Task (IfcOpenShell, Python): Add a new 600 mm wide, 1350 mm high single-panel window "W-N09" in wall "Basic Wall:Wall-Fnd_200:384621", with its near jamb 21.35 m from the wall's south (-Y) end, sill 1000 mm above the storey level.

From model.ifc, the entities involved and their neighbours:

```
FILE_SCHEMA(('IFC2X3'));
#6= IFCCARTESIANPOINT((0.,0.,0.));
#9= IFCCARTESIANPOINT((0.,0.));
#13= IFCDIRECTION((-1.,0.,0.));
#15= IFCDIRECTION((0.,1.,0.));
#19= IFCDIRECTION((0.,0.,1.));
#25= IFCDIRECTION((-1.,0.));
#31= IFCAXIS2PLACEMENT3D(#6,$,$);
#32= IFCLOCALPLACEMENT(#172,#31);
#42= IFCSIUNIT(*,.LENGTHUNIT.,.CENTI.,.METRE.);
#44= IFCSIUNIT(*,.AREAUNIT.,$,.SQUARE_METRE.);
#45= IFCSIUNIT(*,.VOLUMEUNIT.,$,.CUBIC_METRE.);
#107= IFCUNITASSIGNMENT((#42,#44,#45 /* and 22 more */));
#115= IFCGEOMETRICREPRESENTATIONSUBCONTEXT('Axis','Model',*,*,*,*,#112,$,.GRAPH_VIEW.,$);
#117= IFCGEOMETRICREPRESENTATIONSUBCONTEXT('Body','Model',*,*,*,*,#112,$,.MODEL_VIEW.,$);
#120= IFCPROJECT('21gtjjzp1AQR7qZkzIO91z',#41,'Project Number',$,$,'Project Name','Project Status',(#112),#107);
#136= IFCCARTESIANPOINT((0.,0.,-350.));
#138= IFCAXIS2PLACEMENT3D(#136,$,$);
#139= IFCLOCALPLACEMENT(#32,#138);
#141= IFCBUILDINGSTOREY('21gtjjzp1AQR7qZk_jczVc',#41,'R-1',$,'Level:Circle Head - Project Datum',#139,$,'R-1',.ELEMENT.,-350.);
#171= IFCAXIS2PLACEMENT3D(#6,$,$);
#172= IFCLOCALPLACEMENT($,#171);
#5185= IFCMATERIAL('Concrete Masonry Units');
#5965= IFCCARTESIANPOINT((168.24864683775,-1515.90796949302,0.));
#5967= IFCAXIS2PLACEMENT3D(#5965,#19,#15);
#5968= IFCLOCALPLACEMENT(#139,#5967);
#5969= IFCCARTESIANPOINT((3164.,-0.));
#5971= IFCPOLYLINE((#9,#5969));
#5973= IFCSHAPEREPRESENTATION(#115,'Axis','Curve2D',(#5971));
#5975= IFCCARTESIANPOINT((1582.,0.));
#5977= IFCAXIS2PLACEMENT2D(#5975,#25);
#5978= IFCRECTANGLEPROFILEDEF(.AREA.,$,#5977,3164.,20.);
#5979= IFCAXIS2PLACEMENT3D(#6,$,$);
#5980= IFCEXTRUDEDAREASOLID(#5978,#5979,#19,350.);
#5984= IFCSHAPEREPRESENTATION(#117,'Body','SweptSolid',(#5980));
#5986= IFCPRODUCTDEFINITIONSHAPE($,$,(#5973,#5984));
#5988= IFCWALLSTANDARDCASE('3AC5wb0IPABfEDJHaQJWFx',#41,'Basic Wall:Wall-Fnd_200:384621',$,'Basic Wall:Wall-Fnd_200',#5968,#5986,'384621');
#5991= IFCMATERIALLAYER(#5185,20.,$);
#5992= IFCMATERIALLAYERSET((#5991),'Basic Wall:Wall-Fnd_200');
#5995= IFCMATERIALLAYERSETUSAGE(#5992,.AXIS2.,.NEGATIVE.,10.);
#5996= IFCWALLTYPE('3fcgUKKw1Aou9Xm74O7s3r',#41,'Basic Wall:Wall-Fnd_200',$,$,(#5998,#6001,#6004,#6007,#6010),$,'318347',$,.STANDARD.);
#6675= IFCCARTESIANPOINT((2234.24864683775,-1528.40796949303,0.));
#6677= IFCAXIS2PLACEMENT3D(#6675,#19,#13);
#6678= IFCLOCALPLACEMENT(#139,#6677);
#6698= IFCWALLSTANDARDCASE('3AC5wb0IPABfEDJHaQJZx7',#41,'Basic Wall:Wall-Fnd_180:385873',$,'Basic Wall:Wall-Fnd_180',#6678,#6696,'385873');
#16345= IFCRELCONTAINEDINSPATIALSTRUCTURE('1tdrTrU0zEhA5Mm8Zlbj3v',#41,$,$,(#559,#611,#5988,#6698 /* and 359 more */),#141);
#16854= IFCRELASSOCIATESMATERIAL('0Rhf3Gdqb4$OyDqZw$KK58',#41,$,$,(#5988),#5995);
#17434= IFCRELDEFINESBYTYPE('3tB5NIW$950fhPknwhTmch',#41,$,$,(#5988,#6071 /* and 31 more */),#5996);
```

```python
import numpy as np
import ifcopenshell
import ifcopenshell.api.feature
import ifcopenshell.api.geometry
import ifcopenshell.api.root
import ifcopenshell.api.spatial
import ifcopenshell.api.type
import ifcopenshell.geom
import ifcopenshell.util.element
import ifcopenshell.util.placement
import ifcopenshell.util.representation
import ifcopenshell.util.shape
import ifcopenshell.util.unit

model = ifcopenshell.open("model.ifc")
unit_scale = ifcopenshell.util.unit.calculate_unit_scale(model)
settings = ifcopenshell.geom.settings()


def volume(element):
    """Net volume in cubic metres, openings subtracted."""
    shape = ifcopenshell.geom.create_shape(settings, element)
    return ifcopenshell.util.shape.get_volume(shape.geometry)


wall = model.by_guid("3AC5wb0IPABfEDJHaQJWFx")
storey = ifcopenshell.util.element.get_container(wall, ifc_class="IfcBuildingStorey")
context = ifcopenshell.util.representation.get_context(model, "Model", "Body", "MODEL_VIEW")
before = volume(wall)

width, height, from_end, sill = 0.6, 1.35, 21.35, 1  # metres

# The wall runs along its own X axis, and the end named is its -X end.
wall_shape = ifcopenshell.geom.create_shape(settings, wall)
x, y, z = ifcopenshell.util.shape.get_vertices(wall_shape.geometry).T
start = x.min() + from_end
face, thickness = float(y.min()), float(y.max() - y.min())
wall_matrix = ifcopenshell.util.placement.get_local_placement(wall.ObjectPlacement)
level = ifcopenshell.util.placement.get_local_placement(storey.ObjectPlacement)[2, 3]


def in_wall(x, y):
    """Placement at x, y metres in the wall's axes, at sill height."""
    matrix = wall_matrix.copy()
    matrix[:, 3] = wall_matrix @ np.array([x / unit_scale, y / unit_scale, 0.0, 1.0])
    matrix[2, 3] = level + sill / unit_scale
    return matrix


# Opening: a box that overshoots both wall faces by 50 mm.
opening = ifcopenshell.api.root.create_entity(model, ifc_class="IfcOpeningElement")
box = ifcopenshell.api.geometry.add_wall_representation(
    model, context=context, length=width, height=height, thickness=thickness + 0.1
)
ifcopenshell.api.geometry.assign_representation(model, product=opening, representation=box)
ifcopenshell.api.geometry.edit_object_placement(model, product=opening, matrix=in_wall(start, face - 0.05), is_si=False)
ifcopenshell.api.feature.add_feature(model, feature=opening, element=wall)

window = ifcopenshell.api.root.create_entity(model, ifc_class="IfcWindow", name="W-N09")
window.OverallWidth, window.OverallHeight = width / unit_scale, height / unit_scale
body = ifcopenshell.api.geometry.add_window_representation(
    model,
    context=context,
    overall_width=window.OverallWidth,
    overall_height=window.OverallHeight,
    partition_type="SINGLE_PANEL",
)
ifcopenshell.api.geometry.assign_representation(model, product=window, representation=body)
ifcopenshell.api.spatial.assign_container(model, products=[window], relating_structure=storey)
fills = ifcopenshell.api.feature.add_filling(model, opening=opening, element=window)
fills.OwnerHistory = window.OwnerHistory  # required in IFC2X3

# IFC2X3 keeps the operation on the window style.
style = ifcopenshell.api.root.create_entity(model, ifc_class="IfcWindowStyle", name="W-N09")
style.OperationType, style.ConstructionType = "SINGLE_PANEL", "NOTDEFINED"
style.ParameterTakesPrecedence = style.Sizeable = False
ifcopenshell.api.type.assign_type(model, related_objects=[window], relating_type=style)

# Centre the window in the wall's thickness.
ifcopenshell.api.geometry.edit_object_placement(model, product=window, matrix=in_wall(start, face), is_si=False)
window_shape = ifcopenshell.geom.create_shape(settings, window)
depth = ifcopenshell.util.shape.get_vertices(window_shape.geometry)[:, 1]
offset = face + thickness / 2 - (depth.min() + depth.max()) / 2
ifcopenshell.api.geometry.edit_object_placement(model, product=window, matrix=in_wall(start, offset), is_si=False)

after = volume(wall)

print(f"wall volume {before:.3f} -> {after:.3f} m3")

model.write("model_rev.ifc")
```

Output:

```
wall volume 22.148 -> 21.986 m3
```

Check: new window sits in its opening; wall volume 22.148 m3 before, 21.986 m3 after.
